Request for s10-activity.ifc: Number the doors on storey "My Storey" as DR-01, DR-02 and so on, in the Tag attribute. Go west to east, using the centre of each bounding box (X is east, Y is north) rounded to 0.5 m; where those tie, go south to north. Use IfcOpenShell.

First a look at what the model holds.

```python
import ifcopenshell
import ifcopenshell.util.element
import ifcopenshell.util.placement

model = ifcopenshell.open("s10-activity.ifc")
print(model.schema)
storey = next(s for s in model.by_type("IfcBuildingStorey") if s.Name == "My Storey")
doors = [e for e in ifcopenshell.util.element.get_decomposition(storey) if e.is_a("IfcDoor")]
for e in sorted(doors, key=lambda e: e.id()):
    origin = ifcopenshell.util.placement.get_local_placement(e.ObjectPlacement)[:3, 3]
    print(e.id(), e.Tag, e.Name, origin.round(2) + 0.0, sep=" | ")
```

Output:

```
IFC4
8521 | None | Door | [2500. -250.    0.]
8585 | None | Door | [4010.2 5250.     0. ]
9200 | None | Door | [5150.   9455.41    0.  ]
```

```python
import ifcopenshell
import ifcopenshell.geom
import ifcopenshell.util.element
import ifcopenshell.util.shape

model = ifcopenshell.open("s10-activity.ifc")
settings = ifcopenshell.geom.settings()
settings.set("use-world-coords", True)


def centre(element):
    shape = ifcopenshell.geom.create_shape(settings, element)
    return ifcopenshell.util.shape.get_bbox_centroid(shape.geometry)


storey = next(s for s in model.by_type("IfcBuildingStorey") if s.Name == "My Storey")
doors = [e for e in ifcopenshell.util.element.get_decomposition(storey) if e.is_a("IfcDoor")]

# Insertion points can sit at a corner or the storey origin, so sort by the geometry (in metres).
centres = {e: centre(e) for e in doors}
doors.sort(key=lambda e: (round(centres[e][0] / 0.5), centres[e][1]))

for i, e in enumerate(doors, start=1):
    number = f"DR-{i:02d}"
    e.Tag = number
    print(e.id(), number)

model.write("s10-activity_edited.ifc")
```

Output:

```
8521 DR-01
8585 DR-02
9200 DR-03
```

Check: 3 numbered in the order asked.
